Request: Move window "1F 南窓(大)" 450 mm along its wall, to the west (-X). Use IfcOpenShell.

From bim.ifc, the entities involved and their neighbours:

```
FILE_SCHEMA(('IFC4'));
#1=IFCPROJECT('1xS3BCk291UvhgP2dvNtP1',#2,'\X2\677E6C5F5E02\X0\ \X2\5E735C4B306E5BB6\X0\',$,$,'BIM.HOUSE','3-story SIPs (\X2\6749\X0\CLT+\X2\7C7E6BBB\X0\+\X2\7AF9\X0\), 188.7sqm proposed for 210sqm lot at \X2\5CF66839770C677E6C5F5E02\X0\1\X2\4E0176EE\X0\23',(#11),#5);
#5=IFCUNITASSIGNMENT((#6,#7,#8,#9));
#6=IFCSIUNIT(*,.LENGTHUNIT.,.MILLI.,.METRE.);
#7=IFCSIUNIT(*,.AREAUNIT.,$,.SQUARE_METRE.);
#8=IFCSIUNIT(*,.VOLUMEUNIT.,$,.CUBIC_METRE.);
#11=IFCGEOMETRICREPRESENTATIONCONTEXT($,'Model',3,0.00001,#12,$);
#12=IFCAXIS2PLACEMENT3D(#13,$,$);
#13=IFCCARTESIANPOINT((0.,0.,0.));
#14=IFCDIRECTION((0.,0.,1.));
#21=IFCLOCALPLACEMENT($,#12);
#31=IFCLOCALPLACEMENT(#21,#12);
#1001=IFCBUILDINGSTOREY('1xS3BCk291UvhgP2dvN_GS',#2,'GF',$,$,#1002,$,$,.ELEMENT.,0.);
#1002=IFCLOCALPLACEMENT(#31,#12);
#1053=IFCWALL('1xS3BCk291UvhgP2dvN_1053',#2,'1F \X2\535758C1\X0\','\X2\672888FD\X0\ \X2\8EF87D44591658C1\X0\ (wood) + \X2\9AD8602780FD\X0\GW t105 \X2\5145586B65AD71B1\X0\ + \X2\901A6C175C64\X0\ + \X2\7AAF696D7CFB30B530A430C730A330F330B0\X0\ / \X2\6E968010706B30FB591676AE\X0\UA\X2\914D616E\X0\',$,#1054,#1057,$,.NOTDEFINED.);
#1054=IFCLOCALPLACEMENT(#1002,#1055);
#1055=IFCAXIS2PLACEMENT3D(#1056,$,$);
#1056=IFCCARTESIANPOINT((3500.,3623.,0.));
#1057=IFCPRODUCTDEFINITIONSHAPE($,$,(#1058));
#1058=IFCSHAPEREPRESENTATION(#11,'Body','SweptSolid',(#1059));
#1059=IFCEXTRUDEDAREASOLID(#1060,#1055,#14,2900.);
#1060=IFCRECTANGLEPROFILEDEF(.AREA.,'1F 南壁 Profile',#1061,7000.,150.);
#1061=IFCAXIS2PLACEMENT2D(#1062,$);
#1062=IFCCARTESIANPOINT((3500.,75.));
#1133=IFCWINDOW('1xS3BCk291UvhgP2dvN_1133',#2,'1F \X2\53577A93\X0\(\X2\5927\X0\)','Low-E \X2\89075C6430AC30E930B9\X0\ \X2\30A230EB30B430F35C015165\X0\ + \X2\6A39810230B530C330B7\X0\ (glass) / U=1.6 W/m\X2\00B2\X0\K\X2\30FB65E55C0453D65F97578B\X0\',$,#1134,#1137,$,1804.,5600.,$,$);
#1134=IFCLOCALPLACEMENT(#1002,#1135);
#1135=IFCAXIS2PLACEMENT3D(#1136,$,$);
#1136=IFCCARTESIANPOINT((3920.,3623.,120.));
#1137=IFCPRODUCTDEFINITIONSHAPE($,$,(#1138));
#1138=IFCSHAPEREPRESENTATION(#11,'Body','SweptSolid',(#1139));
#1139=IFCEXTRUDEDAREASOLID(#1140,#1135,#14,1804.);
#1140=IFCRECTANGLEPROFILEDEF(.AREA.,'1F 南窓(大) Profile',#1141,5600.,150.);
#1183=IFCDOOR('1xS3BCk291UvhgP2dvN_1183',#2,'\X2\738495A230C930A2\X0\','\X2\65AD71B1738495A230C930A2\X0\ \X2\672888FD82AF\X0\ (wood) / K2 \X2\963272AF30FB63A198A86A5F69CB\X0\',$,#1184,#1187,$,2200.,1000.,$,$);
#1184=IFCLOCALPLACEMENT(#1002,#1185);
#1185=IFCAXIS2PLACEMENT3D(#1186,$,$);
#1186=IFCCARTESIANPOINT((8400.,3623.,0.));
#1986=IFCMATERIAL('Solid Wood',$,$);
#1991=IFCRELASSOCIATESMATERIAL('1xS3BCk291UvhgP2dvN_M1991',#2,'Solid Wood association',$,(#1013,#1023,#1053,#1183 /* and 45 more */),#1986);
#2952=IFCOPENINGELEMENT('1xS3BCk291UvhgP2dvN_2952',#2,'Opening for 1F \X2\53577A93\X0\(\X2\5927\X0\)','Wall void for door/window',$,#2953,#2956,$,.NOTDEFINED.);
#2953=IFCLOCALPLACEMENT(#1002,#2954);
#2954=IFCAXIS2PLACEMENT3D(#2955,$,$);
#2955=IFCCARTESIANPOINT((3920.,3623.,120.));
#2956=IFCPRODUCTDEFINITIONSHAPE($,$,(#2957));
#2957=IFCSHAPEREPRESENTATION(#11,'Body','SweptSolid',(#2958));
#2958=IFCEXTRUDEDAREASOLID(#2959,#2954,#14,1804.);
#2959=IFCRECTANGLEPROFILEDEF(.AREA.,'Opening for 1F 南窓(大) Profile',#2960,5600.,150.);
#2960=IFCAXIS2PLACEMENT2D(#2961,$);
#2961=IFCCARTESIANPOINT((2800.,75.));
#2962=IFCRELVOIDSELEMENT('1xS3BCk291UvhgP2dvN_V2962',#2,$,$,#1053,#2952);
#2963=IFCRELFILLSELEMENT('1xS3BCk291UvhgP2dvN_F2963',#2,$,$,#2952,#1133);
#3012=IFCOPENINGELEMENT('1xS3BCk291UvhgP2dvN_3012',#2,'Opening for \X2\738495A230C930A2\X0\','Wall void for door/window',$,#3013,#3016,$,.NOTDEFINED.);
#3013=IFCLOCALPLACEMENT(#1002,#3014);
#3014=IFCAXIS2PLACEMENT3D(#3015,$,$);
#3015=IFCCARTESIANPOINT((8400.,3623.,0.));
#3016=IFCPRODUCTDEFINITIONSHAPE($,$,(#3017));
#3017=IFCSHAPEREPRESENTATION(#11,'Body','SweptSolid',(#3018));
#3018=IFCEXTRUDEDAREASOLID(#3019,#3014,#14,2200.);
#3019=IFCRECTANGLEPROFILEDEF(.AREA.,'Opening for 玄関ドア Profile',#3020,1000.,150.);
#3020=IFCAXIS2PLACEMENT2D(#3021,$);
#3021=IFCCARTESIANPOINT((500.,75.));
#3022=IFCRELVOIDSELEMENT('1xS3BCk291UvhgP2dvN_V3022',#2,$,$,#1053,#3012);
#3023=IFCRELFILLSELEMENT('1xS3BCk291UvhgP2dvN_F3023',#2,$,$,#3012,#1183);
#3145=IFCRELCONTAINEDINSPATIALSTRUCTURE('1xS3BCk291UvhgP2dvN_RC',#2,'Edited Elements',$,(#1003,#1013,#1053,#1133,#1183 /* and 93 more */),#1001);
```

```python
import ifcopenshell
import ifcopenshell.api.geometry
import ifcopenshell.util.placement

model = ifcopenshell.open("bim.ifc")

window = model.by_guid("1xS3BCk291UvhgP2dvN_1133")
opening = window.FillsVoids[0].RelatingOpeningElement
wall = opening.VoidsElements[0].RelatingBuildingElement

wall_matrix = ifcopenshell.util.placement.get_local_placement(wall.ObjectPlacement)
shift = wall_matrix[:3, 0] * -450.0
before = ifcopenshell.util.placement.get_local_placement(window.ObjectPlacement)[:3, 3].copy()

# The window is not placed relative to its opening, so move both.
for product in (opening, window):
    matrix = ifcopenshell.util.placement.get_local_placement(product.ObjectPlacement)
    matrix[:3, 3] += shift
    ifcopenshell.api.geometry.edit_object_placement(model, product=product, matrix=matrix, is_si=False)

after = ifcopenshell.util.placement.get_local_placement(window.ObjectPlacement)[:3, 3]
print("window moved by", (after - before).round(3) + 0.0)

model.write("bim_edited.ifc")
```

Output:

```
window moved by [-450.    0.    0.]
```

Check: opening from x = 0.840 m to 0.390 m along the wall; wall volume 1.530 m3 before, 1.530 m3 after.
